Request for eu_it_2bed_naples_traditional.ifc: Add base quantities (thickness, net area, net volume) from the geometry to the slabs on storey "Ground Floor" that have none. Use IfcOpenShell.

First a look at what the model holds.

```python
import ifcopenshell
import ifcopenshell.util.element
import ifcopenshell.util.unit

model = ifcopenshell.open("eu_it_2bed_naples_traditional.ifc")
print(model.schema)
for unit_type in ("LENGTHUNIT", "AREAUNIT", "VOLUMEUNIT"):
    print(unit_type, ifcopenshell.util.unit.calculate_unit_scale(model, unit_type))
storey = next(s for s in model.by_type("IfcBuildingStorey") if s.Name == "Ground Floor")
slabs = [e for e in ifcopenshell.util.element.get_decomposition(storey) if e.is_a("IfcSlab")]
for e in sorted(slabs, key=lambda e: e.id()):
    print(e.id(), e.is_a(), e.Name, list(ifcopenshell.util.element.get_psets(e, qtos_only=True)), sep=" | ")
```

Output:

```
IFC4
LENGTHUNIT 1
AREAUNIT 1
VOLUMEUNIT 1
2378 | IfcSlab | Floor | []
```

```python
import ifcopenshell
import ifcopenshell.api.pset
import ifcopenshell.geom
import ifcopenshell.util.element
import ifcopenshell.util.shape
import ifcopenshell.util.unit

model = ifcopenshell.open("eu_it_2bed_naples_traditional.ifc")
unit_scale = ifcopenshell.util.unit.calculate_unit_scale(model)
area_scale = ifcopenshell.util.unit.calculate_unit_scale(model, "AREAUNIT")
volume_scale = ifcopenshell.util.unit.calculate_unit_scale(model, "VOLUMEUNIT")
settings = ifcopenshell.geom.settings()

storey = next(s for s in model.by_type("IfcBuildingStorey") if s.Name == "Ground Floor")
slabs = [e for e in ifcopenshell.util.element.get_decomposition(storey) if e.is_a("IfcSlab")]

for e in sorted(slabs, key=lambda e: e.id()):
    if ifcopenshell.util.element.get_psets(e, qtos_only=True, should_inherit=False):
        continue
    # Geometry comes back in metres, in the element's own axes.
    shape = ifcopenshell.geom.create_shape(settings, e)
    values = {
        "Width": ifcopenshell.util.shape.get_z(shape.geometry) / unit_scale,
        "NetArea": ifcopenshell.util.shape.get_footprint_area(shape.geometry) / area_scale,
        "NetVolume": ifcopenshell.util.shape.get_volume(shape.geometry) / volume_scale,
    }
    qto = ifcopenshell.api.pset.add_qto(model, product=e, name="Qto_SlabBaseQuantities")
    ifcopenshell.api.pset.edit_qto(model, qto=qto, properties=values)
    print(e.id(), {k: round(v, 3) for k, v in values.items()})

model.write("eu_it_2bed_naples_traditional_v2.ifc")
```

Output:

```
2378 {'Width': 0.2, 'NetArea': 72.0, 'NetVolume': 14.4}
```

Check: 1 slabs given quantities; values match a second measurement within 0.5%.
